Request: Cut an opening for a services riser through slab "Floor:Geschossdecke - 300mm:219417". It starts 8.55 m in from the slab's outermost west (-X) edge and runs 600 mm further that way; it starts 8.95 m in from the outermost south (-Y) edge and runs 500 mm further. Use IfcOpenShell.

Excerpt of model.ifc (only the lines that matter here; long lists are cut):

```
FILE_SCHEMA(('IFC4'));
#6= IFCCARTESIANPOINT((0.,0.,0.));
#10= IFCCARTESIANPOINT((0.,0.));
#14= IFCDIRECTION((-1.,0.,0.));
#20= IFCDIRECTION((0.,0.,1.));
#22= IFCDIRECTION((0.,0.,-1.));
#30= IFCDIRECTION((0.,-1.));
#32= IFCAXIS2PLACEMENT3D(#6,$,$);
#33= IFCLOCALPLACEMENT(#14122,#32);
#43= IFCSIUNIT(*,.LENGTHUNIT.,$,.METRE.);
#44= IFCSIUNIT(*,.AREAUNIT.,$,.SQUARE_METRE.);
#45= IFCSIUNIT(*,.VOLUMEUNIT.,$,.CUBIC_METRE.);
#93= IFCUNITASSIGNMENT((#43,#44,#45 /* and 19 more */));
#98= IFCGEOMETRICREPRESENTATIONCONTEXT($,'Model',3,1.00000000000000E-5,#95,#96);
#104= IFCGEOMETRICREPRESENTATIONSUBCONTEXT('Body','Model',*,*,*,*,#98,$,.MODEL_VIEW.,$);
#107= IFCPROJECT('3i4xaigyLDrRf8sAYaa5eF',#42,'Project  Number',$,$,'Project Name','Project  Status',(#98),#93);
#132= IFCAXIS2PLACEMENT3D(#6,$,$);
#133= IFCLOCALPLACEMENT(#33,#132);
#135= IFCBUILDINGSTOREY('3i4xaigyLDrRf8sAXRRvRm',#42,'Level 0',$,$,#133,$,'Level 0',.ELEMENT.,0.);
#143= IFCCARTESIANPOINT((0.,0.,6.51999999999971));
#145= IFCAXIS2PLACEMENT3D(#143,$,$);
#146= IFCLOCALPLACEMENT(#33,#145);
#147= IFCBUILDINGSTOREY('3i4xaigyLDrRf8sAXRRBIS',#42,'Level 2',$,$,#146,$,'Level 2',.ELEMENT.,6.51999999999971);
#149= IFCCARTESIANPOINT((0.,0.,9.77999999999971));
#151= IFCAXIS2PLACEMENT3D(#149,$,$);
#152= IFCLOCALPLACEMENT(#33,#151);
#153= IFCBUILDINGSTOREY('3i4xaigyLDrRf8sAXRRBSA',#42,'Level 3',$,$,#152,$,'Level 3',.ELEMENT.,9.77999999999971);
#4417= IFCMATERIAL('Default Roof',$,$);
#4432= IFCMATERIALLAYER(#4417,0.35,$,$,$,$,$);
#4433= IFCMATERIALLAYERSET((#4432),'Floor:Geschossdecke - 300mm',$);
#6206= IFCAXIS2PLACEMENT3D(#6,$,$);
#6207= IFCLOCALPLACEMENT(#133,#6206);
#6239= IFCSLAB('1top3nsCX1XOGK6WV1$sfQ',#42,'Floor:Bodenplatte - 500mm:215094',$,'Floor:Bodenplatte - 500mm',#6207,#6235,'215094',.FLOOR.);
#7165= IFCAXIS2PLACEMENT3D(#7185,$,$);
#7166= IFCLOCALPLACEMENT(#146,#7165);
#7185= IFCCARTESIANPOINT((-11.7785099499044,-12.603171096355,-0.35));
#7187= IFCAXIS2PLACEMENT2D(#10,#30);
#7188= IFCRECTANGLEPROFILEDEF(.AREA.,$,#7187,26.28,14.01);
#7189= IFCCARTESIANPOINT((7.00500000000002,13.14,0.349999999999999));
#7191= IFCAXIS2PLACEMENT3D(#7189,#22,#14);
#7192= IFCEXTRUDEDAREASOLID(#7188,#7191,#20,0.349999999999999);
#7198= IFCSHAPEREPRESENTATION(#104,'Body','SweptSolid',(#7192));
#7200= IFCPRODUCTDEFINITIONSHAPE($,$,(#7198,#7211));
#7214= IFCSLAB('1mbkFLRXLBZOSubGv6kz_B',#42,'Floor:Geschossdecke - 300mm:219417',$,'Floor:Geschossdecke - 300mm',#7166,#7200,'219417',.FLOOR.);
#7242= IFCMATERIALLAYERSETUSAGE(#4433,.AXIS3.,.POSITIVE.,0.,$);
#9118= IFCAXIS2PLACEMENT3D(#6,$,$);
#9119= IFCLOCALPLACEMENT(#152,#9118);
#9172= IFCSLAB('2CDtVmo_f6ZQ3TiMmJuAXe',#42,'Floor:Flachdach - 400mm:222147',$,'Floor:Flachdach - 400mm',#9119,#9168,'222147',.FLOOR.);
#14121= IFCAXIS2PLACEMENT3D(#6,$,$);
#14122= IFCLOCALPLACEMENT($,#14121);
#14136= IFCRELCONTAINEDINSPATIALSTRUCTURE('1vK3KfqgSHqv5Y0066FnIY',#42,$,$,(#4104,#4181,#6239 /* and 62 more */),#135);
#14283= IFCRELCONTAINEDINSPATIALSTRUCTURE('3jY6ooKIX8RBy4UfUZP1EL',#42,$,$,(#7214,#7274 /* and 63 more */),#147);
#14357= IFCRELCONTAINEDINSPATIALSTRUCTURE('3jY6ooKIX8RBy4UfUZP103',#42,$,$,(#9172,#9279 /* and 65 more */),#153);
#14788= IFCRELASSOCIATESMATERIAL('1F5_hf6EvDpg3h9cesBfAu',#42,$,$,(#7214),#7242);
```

```python
import numpy as np
import ifcopenshell
import ifcopenshell.api.feature
import ifcopenshell.api.geometry
import ifcopenshell.api.root
import ifcopenshell.geom
import ifcopenshell.util.placement
import ifcopenshell.util.representation
import ifcopenshell.util.shape
import ifcopenshell.util.unit

model = ifcopenshell.open("model.ifc")
unit_scale = ifcopenshell.util.unit.calculate_unit_scale(model)
settings = ifcopenshell.geom.settings()


def volume(element):
    """Net volume in cubic metres, openings subtracted."""
    shape = ifcopenshell.geom.create_shape(settings, element)
    return ifcopenshell.util.shape.get_volume(shape.geometry)


slab = model.by_id(7214)
before = volume(slab)

# Extent in the slab's own axes, in metres. The edges named are its -X and -Y sides.
slab_shape = ifcopenshell.geom.create_shape(settings, slab)
vertices = ifcopenshell.util.shape.get_vertices(slab_shape.geometry)
x_min, y_min, bottom = vertices.min(axis=0)
top = vertices[:, 2].max()

opening = ifcopenshell.api.root.create_entity(model, ifc_class="IfcOpeningElement", name="Services riser opening", predefined_type="OPENING")
context = ifcopenshell.util.representation.get_context(model, "Model", "Body", "MODEL_VIEW")
width, depth = 0.6, 0.5
outline = [(0.0, 0.0), (width, 0.0), (width, depth), (0.0, depth), (0.0, 0.0)]
# Overshoot both faces by 50 mm so the cut is clean.
shape = ifcopenshell.api.geometry.add_slab_representation(
    model, context=context, depth=top - bottom + 0.1, polyline=outline
)
ifcopenshell.api.geometry.assign_representation(model, product=opening, representation=shape)

matrix = ifcopenshell.util.placement.get_local_placement(slab.ObjectPlacement)
matrix[:, 3] = matrix @ np.append(np.array([x_min + 8.55, y_min + 8.95, bottom - 0.05]) / unit_scale, 1.0)
ifcopenshell.api.geometry.edit_object_placement(model, product=opening, matrix=matrix, is_si=False)
ifcopenshell.api.feature.add_feature(model, feature=opening, element=slab)

after = volume(slab)

print(f"slab volume {before:.3f} -> {after:.3f} m3")

model.write("model_updated.ifc")
```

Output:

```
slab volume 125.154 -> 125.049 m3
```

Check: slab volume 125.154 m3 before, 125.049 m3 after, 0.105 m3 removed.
